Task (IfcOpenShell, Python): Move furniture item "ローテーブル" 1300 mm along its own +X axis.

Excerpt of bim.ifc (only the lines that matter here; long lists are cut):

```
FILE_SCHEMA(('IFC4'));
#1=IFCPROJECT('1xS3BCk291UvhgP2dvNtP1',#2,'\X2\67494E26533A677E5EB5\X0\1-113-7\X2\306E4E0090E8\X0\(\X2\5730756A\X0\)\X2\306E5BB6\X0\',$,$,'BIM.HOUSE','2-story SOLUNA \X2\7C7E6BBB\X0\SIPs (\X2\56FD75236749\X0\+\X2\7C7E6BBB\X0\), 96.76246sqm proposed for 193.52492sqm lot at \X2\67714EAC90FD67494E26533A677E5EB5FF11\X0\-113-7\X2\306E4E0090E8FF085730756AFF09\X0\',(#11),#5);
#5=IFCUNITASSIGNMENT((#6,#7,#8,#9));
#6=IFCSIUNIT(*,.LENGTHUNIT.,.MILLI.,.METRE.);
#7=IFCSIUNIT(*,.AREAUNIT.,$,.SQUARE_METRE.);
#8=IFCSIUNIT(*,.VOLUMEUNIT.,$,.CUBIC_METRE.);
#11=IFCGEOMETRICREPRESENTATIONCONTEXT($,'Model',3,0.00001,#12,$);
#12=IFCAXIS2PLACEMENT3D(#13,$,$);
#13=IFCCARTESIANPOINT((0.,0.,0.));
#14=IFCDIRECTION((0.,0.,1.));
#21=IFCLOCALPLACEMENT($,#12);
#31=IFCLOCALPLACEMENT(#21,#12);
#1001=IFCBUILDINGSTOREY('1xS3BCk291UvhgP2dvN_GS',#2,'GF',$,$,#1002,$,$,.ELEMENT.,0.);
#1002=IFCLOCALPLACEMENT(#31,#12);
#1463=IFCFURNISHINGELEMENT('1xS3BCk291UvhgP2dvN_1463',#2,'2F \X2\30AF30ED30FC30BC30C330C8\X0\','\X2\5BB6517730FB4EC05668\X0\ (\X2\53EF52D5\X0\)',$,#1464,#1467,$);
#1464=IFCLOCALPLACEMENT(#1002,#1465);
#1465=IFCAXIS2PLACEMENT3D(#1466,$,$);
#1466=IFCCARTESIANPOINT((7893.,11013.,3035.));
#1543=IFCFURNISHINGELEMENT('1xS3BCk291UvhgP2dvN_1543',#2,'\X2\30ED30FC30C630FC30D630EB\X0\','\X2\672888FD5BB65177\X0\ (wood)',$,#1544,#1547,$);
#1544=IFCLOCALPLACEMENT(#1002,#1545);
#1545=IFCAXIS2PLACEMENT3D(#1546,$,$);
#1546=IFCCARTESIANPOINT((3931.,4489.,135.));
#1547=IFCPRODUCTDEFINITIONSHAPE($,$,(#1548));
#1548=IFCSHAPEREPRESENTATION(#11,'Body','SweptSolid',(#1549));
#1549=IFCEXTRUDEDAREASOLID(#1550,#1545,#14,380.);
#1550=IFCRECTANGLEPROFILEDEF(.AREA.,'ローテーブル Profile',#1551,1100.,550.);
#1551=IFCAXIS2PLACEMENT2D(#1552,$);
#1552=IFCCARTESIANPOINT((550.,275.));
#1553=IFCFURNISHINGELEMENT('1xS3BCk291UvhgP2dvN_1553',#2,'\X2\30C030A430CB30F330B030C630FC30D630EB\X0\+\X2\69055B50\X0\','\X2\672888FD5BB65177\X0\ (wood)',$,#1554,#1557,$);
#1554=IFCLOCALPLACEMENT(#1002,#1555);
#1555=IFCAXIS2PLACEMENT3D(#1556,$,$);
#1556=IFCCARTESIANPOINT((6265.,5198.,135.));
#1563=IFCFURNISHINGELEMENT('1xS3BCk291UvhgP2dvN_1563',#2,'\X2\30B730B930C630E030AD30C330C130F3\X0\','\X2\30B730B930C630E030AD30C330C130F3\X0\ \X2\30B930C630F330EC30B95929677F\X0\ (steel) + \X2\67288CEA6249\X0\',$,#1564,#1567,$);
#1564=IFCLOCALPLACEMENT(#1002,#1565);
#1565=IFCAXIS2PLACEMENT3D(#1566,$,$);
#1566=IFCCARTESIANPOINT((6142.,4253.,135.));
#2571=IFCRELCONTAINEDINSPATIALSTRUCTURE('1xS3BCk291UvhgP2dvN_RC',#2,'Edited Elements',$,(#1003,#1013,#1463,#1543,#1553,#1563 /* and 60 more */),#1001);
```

```python
import ifcopenshell
import ifcopenshell.api.geometry
import ifcopenshell.util.placement
import ifcopenshell.util.unit

model = ifcopenshell.open("bim.ifc")
unit_scale = ifcopenshell.util.unit.calculate_unit_scale(model)

item = model.by_guid("1xS3BCk291UvhgP2dvN_1543")
matrix = ifcopenshell.util.placement.get_local_placement(item.ObjectPlacement)
matrix[:3, 3] += matrix[:3, 0] * 1.3 / unit_scale
ifcopenshell.api.geometry.edit_object_placement(model, product=item, matrix=matrix, is_si=False)

print(ifcopenshell.util.placement.get_local_placement(item.ObjectPlacement).round(3) + 0.0)

model.write("bim_updated.ifc")
```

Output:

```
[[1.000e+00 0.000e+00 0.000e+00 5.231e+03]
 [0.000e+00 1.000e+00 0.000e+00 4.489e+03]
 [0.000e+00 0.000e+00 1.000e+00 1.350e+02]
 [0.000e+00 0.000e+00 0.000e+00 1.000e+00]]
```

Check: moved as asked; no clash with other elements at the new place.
